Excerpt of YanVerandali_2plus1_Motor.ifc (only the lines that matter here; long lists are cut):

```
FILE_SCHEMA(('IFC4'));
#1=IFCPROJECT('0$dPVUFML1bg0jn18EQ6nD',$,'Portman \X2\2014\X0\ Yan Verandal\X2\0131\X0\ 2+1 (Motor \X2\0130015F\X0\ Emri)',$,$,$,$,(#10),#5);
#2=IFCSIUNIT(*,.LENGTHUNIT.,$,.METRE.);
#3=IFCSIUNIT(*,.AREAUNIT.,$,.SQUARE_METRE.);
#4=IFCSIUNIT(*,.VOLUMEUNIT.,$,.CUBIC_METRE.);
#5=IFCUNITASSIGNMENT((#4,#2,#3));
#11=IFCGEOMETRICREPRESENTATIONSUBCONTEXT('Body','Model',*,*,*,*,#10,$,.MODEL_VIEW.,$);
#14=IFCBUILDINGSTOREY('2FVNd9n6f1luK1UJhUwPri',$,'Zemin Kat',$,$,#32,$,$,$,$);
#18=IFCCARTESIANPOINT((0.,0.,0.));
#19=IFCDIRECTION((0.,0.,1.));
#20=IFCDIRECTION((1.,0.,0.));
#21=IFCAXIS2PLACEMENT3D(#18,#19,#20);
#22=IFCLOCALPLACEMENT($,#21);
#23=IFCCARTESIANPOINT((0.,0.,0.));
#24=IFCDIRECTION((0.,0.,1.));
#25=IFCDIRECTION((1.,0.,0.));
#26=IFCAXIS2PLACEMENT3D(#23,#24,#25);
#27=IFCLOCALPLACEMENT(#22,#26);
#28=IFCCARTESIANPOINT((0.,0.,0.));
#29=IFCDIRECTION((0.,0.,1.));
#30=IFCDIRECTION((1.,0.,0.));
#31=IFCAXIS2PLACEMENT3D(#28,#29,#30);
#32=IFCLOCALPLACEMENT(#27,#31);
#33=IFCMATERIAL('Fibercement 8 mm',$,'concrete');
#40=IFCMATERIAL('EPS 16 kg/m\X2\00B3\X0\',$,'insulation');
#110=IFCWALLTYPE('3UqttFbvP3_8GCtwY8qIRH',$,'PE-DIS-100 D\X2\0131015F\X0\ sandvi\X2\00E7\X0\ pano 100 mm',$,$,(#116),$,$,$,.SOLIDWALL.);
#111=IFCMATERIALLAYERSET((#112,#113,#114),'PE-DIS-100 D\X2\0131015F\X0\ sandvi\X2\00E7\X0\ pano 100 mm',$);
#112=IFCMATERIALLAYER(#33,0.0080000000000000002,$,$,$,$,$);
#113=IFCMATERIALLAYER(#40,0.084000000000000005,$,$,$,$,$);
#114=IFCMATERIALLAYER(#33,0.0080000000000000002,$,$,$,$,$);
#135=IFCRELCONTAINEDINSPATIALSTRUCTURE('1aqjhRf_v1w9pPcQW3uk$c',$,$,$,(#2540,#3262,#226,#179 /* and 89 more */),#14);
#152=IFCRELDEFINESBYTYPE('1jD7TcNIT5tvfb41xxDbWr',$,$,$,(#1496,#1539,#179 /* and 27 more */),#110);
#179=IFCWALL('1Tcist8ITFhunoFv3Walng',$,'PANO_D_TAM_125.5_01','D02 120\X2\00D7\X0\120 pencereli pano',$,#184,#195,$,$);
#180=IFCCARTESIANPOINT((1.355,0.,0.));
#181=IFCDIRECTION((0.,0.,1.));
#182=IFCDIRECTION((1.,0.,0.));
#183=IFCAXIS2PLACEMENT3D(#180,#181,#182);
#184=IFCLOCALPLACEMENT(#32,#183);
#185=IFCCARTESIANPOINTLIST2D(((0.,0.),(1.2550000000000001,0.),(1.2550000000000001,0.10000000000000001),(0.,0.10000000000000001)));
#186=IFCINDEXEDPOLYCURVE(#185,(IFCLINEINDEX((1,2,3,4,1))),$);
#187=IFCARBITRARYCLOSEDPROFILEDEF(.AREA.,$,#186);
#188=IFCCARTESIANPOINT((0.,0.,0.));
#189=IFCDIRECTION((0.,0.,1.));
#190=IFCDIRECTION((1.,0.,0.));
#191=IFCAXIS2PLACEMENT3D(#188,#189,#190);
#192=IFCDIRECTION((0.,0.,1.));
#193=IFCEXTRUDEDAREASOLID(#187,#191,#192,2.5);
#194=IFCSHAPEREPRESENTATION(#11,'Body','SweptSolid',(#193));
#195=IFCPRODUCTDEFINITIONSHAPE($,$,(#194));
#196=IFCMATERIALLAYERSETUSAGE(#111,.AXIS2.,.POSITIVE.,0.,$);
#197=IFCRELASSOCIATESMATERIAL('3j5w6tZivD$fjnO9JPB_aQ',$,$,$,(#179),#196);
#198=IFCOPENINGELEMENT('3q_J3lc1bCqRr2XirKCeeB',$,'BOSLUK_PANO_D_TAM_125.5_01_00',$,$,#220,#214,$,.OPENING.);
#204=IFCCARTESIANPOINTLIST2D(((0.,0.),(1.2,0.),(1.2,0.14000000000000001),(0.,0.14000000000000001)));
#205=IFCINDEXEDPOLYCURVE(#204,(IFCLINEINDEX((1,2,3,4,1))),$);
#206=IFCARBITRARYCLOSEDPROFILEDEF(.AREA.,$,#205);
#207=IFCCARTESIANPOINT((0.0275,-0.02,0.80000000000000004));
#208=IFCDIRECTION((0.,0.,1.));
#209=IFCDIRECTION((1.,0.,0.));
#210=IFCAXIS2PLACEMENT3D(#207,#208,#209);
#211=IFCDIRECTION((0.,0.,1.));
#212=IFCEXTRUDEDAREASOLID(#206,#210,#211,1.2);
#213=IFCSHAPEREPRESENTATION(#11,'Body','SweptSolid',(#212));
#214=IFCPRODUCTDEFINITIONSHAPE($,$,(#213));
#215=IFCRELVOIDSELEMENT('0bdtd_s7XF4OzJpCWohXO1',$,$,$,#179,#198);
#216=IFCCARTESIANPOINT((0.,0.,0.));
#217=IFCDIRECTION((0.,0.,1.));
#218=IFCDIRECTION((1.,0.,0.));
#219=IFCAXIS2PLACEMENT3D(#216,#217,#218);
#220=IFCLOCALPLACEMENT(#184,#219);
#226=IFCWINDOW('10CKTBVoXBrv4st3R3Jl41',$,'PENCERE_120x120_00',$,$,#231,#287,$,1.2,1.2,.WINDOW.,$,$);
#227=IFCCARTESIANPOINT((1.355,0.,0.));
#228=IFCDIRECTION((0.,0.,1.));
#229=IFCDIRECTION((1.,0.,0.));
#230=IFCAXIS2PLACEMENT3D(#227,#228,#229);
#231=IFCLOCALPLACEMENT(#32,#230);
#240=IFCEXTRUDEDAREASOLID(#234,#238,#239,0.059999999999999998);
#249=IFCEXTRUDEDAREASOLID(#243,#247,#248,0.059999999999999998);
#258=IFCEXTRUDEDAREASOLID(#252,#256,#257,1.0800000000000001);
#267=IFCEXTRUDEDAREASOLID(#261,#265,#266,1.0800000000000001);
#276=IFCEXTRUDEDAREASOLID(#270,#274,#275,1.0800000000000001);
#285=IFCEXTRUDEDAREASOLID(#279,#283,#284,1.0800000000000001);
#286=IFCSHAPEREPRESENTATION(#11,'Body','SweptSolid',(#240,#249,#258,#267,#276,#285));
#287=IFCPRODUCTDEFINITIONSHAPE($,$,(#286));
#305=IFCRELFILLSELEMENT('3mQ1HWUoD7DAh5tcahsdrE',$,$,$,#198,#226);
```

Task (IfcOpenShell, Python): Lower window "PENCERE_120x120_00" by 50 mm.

```python
import numpy as np
import ifcopenshell
import ifcopenshell.api.geometry
import ifcopenshell.util.placement
import ifcopenshell.util.unit

model = ifcopenshell.open("YanVerandali_2plus1_Motor.ifc")
unit_scale = ifcopenshell.util.unit.calculate_unit_scale(model)

window = model.by_id(226)
opening = window.FillsVoids[0].RelatingOpeningElement
dz = -0.05 / unit_scale

shift = np.array([0.0, 0.0, dz])
# The window is not placed relative to its opening, so move both.
for product in (opening, window):
    matrix = ifcopenshell.util.placement.get_local_placement(product.ObjectPlacement)
    matrix[:3, 3] += shift
    ifcopenshell.api.geometry.edit_object_placement(model, product=product, matrix=matrix, is_si=False)

print(f"moved by {dz * unit_scale:+.3f} m")

model.write("YanVerandali_2plus1_Motor_updated.ifc")
```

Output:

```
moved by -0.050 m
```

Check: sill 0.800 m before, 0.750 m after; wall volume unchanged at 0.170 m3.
